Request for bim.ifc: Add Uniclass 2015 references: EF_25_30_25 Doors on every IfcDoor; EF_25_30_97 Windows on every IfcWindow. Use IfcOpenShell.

First a look at what the model holds.

```python
import ifcopenshell

model = ifcopenshell.open("bim.ifc")
print(model.schema)
print("classifications:", [c.Name for c in model.by_type("IfcClassification")])
for ifc_class in ("IfcDoor", "IfcRoof", "IfcStair", "IfcWall", "IfcWindow"):
    print(ifc_class, len(model.by_type(ifc_class)))
```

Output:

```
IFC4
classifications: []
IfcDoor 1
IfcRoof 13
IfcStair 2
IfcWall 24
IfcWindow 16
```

```python
import ifcopenshell
import ifcopenshell.api.classification

model = ifcopenshell.open("bim.ifc")

system = ifcopenshell.api.classification.add_classification(model, classification="Uniclass 2015")

codes = {
    "IfcDoor": ("EF_25_30_25", "Doors"),
    "IfcWindow": ("EF_25_30_97", "Windows"),
}
for ifc_class, (code, name) in codes.items():
    products = model.by_type(ifc_class)
    ifcopenshell.api.classification.add_reference(
        model, products=products, classification=system, identification=code, name=name
    )
    print(code, len(products))

model.write("bim-out.ifc")
```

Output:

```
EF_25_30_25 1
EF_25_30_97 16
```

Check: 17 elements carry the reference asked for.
